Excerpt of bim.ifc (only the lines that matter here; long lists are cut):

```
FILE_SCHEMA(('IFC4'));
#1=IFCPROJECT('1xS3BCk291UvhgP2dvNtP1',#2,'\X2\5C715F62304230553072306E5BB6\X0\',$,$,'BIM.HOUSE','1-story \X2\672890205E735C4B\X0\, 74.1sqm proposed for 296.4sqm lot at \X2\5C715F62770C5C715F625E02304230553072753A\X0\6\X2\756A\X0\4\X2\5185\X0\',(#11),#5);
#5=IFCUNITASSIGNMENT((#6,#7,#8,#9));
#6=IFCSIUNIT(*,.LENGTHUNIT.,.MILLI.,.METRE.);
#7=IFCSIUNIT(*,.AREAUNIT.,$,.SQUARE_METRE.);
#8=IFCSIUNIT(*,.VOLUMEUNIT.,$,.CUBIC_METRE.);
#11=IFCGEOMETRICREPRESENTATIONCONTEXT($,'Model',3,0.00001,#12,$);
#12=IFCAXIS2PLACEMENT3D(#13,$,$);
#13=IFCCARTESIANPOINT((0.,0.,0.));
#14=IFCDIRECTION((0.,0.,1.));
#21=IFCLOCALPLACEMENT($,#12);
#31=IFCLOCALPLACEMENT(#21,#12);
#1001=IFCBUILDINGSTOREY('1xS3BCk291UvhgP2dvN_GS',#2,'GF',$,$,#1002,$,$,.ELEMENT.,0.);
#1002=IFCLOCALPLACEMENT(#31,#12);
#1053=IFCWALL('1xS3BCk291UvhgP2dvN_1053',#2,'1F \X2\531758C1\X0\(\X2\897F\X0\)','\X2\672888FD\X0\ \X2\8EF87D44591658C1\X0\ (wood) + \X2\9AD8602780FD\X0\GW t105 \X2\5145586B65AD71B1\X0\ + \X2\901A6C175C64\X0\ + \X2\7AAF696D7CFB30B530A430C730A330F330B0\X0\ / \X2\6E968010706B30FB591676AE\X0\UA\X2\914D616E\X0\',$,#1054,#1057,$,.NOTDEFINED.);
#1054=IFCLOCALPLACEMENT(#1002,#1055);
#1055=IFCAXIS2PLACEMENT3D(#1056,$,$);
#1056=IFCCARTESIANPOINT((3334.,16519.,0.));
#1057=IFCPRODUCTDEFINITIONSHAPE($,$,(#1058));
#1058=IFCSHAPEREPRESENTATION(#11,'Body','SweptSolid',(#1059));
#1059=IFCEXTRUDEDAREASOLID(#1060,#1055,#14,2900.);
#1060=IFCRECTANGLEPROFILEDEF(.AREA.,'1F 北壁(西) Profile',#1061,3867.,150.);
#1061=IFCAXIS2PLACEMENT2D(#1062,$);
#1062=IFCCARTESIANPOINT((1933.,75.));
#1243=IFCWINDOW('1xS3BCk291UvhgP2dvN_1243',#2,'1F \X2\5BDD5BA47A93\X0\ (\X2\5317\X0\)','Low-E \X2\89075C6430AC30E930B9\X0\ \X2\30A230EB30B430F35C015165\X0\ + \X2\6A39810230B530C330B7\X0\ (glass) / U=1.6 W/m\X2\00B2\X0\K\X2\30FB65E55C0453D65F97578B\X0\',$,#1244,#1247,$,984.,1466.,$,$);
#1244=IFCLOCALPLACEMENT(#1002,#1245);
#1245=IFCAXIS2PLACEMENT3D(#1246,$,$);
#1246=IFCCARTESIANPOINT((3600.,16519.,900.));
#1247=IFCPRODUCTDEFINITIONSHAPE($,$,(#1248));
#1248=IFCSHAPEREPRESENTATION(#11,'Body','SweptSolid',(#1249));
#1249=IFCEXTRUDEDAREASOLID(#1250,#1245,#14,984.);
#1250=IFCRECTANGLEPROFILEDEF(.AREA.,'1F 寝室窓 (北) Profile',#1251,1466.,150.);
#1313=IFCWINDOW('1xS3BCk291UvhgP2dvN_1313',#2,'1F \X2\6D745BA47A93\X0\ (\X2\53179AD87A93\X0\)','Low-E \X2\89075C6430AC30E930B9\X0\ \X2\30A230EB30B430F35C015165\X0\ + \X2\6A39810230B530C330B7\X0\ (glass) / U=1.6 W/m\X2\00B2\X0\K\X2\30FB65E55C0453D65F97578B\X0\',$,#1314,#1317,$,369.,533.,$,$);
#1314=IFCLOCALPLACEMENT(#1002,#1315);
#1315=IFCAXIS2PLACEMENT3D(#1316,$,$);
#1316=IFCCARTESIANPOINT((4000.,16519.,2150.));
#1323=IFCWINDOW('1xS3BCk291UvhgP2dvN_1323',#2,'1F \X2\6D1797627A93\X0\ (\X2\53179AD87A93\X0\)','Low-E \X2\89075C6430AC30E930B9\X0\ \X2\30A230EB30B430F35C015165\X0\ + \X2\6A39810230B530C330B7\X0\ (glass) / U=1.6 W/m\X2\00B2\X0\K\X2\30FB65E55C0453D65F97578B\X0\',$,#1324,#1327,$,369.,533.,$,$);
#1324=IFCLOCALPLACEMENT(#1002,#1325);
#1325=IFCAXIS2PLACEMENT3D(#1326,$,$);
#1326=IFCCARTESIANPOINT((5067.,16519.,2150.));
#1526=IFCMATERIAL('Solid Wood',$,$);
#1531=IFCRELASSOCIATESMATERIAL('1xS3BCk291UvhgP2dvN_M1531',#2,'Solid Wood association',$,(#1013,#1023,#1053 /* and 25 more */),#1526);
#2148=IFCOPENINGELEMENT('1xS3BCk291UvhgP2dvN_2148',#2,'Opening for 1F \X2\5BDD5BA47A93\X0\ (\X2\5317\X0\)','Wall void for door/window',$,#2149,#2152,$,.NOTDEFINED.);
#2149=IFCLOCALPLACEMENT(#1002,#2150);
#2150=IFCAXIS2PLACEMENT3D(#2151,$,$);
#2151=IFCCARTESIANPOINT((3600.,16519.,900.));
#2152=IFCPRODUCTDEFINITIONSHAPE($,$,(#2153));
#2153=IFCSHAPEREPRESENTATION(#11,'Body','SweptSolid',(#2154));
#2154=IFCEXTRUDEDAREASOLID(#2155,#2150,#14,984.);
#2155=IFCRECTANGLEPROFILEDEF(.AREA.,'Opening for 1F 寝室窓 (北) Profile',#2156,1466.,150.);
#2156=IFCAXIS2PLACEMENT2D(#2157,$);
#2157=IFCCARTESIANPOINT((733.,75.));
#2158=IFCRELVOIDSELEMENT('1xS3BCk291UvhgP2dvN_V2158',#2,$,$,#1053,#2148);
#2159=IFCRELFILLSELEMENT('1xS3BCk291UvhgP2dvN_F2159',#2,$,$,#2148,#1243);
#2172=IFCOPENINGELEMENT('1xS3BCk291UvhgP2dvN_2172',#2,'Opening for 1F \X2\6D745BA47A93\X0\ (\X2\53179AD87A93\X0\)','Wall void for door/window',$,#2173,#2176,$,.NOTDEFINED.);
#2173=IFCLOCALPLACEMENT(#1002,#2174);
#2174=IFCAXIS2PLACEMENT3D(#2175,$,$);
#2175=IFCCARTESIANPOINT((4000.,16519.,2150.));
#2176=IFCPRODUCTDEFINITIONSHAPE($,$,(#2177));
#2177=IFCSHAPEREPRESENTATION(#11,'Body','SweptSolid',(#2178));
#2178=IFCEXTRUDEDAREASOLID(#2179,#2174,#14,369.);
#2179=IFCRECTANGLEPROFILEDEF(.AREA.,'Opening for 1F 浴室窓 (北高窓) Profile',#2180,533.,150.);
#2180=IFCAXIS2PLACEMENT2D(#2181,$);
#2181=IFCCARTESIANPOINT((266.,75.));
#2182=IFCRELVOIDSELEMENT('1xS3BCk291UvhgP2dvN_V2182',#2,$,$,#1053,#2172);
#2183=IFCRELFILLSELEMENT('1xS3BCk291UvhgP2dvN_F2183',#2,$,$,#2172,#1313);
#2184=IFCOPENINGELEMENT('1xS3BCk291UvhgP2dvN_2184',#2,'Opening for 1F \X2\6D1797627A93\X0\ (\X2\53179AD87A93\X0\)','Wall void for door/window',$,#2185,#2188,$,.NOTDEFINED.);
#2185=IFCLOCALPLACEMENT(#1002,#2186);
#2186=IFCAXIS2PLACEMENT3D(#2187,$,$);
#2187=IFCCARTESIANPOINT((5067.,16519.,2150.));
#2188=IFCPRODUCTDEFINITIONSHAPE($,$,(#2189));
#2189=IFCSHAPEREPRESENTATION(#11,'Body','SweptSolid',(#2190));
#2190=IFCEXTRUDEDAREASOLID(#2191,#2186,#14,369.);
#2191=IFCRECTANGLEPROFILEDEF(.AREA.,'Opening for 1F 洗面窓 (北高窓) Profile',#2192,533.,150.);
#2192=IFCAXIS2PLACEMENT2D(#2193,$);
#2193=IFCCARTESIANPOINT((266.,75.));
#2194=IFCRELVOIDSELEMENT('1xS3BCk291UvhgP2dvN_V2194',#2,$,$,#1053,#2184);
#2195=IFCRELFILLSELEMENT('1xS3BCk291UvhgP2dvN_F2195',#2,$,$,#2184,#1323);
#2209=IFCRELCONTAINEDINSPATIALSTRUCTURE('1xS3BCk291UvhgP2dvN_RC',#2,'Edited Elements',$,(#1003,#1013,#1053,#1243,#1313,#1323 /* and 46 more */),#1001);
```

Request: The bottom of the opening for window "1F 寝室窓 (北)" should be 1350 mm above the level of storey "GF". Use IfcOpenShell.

```python
import numpy as np
import ifcopenshell
import ifcopenshell.api.geometry
import ifcopenshell.geom
import ifcopenshell.util.element
import ifcopenshell.util.placement
import ifcopenshell.util.shape
import ifcopenshell.util.unit

model = ifcopenshell.open("bim.ifc")
unit_scale = ifcopenshell.util.unit.calculate_unit_scale(model)

window = model.by_guid("1xS3BCk291UvhgP2dvN_1243")
opening = window.FillsVoids[0].RelatingOpeningElement
storey = ifcopenshell.util.element.get_container(window, ifc_class="IfcBuildingStorey")
level = ifcopenshell.util.placement.get_local_placement(storey.ObjectPlacement)[2, 3]

# The opening's origin need not be at the sill, so measure its lowest point.
shape = ifcopenshell.geom.create_shape(ifcopenshell.geom.settings(), opening)
bottom = ifcopenshell.util.shape.get_shape_bottom_elevation(shape, shape.geometry) / unit_scale
dz = level + 1350.0 - bottom

shift = np.array([0.0, 0.0, dz])
# The window is not placed relative to its opening, so move both.
for product in (opening, window):
    matrix = ifcopenshell.util.placement.get_local_placement(product.ObjectPlacement)
    matrix[:3, 3] += shift
    ifcopenshell.api.geometry.edit_object_placement(model, product=product, matrix=matrix, is_si=False)

print(f"moved by {dz * unit_scale:+.3f} m")

model.write("bim_rev.ifc")
```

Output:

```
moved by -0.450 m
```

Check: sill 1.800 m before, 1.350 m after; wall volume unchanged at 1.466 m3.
